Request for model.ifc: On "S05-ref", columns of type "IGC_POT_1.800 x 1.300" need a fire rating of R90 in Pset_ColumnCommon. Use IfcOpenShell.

First a look at what the model holds.

```python
import ifcopenshell
import ifcopenshell.util.element

model = ifcopenshell.open("model.ifc")
print(model.schema)
storey = next(s for s in model.by_type("IfcBuildingStorey") if s.Name == "S05-ref")
columns = [e for e in ifcopenshell.util.element.get_decomposition(storey) if e.is_a("IfcColumn")]
seen = {}
for e in columns:
    element_type = ifcopenshell.util.element.get_type(e)
    key = (element_type.Name if element_type != e and element_type else None, ifcopenshell.util.element.get_pset(e, "Pset_ColumnCommon", "FireRating"))
    seen[key] = seen.get(key, 0) + 1
for (name, value), count in sorted(seen.items(), key=str):
    print(count, "x", name, "|", value)
```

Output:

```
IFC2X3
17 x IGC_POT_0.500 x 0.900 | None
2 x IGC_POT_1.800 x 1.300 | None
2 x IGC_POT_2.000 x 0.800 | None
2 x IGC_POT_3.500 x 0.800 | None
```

```python
import ifcopenshell
import ifcopenshell.api.pset
import ifcopenshell.util.element

model = ifcopenshell.open("model.ifc")

storey = next(s for s in model.by_type("IfcBuildingStorey") if s.Name == "S05-ref")
columns = [e for e in ifcopenshell.util.element.get_decomposition(storey) if e.is_a("IfcColumn")]

count = 0
for e in columns:
    element_type = ifcopenshell.util.element.get_type(e)
    if element_type in (None, e) or element_type.Name != "IGC_POT_1.800 x 1.300":
        continue
    # add_pset returns the element's existing set when there is one.
    pset = ifcopenshell.api.pset.add_pset(model, product=e, name="Pset_ColumnCommon")
    ifcopenshell.api.pset.edit_pset(model, pset=pset, properties={"FireRating": "R90"})
    count += 1

print(count, "columns updated")

model.write("model_v2.ifc")
```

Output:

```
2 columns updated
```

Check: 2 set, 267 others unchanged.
